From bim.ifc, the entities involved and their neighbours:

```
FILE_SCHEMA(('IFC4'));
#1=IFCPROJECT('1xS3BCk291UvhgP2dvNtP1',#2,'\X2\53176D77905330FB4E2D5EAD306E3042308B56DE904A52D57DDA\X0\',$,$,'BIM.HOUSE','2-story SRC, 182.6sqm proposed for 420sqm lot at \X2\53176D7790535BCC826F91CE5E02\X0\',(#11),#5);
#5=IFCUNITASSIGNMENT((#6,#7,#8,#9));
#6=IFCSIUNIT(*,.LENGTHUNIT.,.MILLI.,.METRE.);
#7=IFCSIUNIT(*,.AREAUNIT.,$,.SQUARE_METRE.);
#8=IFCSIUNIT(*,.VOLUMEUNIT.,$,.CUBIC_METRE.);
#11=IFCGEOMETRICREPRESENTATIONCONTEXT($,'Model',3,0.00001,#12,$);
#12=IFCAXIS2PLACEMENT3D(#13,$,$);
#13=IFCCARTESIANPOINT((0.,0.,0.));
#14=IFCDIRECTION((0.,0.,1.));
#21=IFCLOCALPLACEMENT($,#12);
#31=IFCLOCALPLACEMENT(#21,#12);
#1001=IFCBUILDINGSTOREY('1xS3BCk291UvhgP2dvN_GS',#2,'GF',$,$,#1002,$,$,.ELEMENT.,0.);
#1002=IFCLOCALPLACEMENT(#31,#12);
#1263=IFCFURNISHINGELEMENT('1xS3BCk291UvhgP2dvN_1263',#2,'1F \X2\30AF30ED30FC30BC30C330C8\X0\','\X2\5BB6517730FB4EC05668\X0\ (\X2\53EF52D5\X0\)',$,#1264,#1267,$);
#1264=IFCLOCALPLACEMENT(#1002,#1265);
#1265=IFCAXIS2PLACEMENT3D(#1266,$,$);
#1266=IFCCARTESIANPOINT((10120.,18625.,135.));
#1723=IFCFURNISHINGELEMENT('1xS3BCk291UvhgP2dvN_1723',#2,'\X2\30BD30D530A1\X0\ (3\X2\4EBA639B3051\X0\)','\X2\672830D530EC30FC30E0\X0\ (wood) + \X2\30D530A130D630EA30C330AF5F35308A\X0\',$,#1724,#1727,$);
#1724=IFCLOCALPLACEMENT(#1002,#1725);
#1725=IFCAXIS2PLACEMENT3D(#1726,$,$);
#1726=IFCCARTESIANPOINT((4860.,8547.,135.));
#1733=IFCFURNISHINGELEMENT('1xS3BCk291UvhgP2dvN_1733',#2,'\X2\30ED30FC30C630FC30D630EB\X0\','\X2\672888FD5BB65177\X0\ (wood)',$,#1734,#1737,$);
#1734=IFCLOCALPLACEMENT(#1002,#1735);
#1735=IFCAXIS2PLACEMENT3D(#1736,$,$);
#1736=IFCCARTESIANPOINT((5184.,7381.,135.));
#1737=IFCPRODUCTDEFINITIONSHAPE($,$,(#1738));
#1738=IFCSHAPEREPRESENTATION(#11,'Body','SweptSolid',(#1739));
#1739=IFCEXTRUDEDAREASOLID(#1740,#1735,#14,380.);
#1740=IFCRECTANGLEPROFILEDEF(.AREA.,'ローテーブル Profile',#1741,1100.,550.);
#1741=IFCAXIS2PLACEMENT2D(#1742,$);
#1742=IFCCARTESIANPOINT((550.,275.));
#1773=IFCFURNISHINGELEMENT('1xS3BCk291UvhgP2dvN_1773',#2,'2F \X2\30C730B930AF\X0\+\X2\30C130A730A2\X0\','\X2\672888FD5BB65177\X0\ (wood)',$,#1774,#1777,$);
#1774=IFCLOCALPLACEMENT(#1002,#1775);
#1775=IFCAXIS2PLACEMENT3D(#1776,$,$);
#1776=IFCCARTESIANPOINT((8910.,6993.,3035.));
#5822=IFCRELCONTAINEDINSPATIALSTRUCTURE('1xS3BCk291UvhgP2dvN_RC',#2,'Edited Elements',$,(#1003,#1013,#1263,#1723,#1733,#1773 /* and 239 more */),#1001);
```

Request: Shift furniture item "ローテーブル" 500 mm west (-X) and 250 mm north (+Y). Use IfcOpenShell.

```python
import ifcopenshell
import ifcopenshell.api.geometry
import ifcopenshell.util.placement
import ifcopenshell.util.unit

model = ifcopenshell.open("bim.ifc")
unit_scale = ifcopenshell.util.unit.calculate_unit_scale(model)

item = model.by_guid("1xS3BCk291UvhgP2dvN_1733")
matrix = ifcopenshell.util.placement.get_local_placement(item.ObjectPlacement)
matrix[0, 3] -= 0.5 / unit_scale
matrix[1, 3] += 0.25 / unit_scale
ifcopenshell.api.geometry.edit_object_placement(model, product=item, matrix=matrix, is_si=False)

print(ifcopenshell.util.placement.get_local_placement(item.ObjectPlacement).round(3) + 0.0)

model.write("bim-out.ifc")
```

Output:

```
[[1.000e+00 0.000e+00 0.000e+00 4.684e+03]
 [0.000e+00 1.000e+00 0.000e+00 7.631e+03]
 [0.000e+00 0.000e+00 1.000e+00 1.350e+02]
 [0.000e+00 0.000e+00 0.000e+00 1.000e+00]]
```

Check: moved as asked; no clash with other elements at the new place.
